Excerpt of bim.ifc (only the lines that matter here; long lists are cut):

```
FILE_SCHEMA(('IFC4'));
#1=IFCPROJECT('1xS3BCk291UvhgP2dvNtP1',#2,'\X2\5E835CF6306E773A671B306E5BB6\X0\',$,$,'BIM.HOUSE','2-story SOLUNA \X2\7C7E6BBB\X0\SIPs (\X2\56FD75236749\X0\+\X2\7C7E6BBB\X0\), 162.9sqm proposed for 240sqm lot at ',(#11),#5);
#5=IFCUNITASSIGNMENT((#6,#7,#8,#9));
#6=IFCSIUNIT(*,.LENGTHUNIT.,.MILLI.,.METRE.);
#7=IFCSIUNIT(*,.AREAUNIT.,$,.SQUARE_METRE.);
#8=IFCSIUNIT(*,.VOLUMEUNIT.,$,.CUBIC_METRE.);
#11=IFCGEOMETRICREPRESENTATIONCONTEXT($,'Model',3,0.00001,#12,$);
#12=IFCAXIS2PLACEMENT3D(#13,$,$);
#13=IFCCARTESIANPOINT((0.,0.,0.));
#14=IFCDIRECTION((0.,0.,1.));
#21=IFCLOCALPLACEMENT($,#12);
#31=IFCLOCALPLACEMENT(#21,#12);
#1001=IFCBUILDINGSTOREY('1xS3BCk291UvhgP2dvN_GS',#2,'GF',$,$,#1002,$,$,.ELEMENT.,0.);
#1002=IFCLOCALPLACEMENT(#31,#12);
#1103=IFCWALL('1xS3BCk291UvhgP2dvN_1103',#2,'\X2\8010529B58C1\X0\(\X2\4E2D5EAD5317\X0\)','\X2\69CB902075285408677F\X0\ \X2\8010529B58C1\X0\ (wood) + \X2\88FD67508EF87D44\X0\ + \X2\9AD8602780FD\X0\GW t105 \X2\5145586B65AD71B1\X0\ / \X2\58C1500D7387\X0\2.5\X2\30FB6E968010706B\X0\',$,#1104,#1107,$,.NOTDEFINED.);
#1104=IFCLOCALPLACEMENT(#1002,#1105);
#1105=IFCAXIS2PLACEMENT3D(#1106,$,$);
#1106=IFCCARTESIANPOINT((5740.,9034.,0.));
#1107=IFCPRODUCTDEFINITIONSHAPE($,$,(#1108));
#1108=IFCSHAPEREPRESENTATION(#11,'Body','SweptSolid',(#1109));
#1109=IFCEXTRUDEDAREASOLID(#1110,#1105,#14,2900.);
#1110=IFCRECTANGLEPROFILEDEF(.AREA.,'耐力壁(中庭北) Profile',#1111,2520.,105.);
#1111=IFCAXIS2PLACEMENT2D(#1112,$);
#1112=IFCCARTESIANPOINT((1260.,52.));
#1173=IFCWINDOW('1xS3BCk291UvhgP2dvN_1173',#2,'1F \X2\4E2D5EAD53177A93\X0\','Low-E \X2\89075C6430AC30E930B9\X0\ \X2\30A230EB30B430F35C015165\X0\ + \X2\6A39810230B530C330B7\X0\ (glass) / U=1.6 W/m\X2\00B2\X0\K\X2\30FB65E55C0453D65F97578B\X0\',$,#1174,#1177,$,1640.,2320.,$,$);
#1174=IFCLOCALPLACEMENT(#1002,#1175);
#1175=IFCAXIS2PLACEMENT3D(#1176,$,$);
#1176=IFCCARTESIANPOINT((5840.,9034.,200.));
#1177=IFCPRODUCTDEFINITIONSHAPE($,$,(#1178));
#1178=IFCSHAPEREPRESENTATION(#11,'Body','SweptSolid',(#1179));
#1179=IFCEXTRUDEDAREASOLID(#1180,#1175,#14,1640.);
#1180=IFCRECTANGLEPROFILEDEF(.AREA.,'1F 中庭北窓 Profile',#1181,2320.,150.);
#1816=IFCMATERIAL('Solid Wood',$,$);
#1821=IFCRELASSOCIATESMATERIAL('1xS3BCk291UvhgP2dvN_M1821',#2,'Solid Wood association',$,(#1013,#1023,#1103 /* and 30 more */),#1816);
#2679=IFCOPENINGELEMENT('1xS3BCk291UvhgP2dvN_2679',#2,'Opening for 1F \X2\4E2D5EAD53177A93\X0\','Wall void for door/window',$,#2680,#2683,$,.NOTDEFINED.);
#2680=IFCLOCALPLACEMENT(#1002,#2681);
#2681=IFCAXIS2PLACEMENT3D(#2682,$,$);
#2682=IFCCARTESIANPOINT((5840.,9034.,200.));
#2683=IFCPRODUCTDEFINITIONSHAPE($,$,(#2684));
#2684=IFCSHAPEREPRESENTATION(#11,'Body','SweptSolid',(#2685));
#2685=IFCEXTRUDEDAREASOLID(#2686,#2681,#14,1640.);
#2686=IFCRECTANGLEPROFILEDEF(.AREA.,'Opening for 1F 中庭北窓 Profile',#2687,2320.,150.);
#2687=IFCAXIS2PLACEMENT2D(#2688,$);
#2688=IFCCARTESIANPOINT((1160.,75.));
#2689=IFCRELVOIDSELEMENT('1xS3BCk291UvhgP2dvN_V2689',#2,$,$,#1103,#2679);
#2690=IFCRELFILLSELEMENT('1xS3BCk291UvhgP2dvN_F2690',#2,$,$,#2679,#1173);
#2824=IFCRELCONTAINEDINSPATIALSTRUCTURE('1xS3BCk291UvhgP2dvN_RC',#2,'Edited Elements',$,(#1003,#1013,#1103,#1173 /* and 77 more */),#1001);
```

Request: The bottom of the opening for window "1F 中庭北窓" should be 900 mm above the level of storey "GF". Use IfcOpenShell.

```python
import numpy as np
import ifcopenshell
import ifcopenshell.api.geometry
import ifcopenshell.geom
import ifcopenshell.util.element
import ifcopenshell.util.placement
import ifcopenshell.util.shape
import ifcopenshell.util.unit

model = ifcopenshell.open("bim.ifc")
unit_scale = ifcopenshell.util.unit.calculate_unit_scale(model)

window = model.by_id(1173)
opening = window.FillsVoids[0].RelatingOpeningElement
storey = ifcopenshell.util.element.get_container(window, ifc_class="IfcBuildingStorey")
level = ifcopenshell.util.placement.get_local_placement(storey.ObjectPlacement)[2, 3]

# The opening's origin need not be at the sill, so measure its lowest point.
shape = ifcopenshell.geom.create_shape(ifcopenshell.geom.settings(), opening)
bottom = ifcopenshell.util.shape.get_shape_bottom_elevation(shape, shape.geometry) / unit_scale
dz = level + 900.0 - bottom

shift = np.array([0.0, 0.0, dz])
# The window is not placed relative to its opening, so move both.
for product in (opening, window):
    matrix = ifcopenshell.util.placement.get_local_placement(product.ObjectPlacement)
    matrix[:3, 3] += shift
    ifcopenshell.api.geometry.edit_object_placement(model, product=product, matrix=matrix, is_si=False)

print(f"moved by {dz * unit_scale:+.3f} m")

model.write("bim-out.ifc")
```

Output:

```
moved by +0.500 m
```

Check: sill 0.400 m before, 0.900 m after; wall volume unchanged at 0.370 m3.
